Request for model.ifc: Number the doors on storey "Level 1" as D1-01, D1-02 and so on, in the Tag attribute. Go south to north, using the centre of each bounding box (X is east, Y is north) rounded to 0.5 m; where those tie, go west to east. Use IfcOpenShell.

First a look at what the model holds.

```python
import ifcopenshell
import ifcopenshell.util.element
import ifcopenshell.util.placement

model = ifcopenshell.open("model.ifc")
print(model.schema)
storey = next(s for s in model.by_type("IfcBuildingStorey") if s.Name == "Level 1")
doors = [e for e in ifcopenshell.util.element.get_decomposition(storey) if e.is_a("IfcDoor")]
for e in sorted(doors, key=lambda e: e.id()):
    origin = ifcopenshell.util.placement.get_local_placement(e.ObjectPlacement)[:3, 3]
    print(e.id(), e.Tag, e.Name, origin.round(2) + 0.0, sep=" | ")
```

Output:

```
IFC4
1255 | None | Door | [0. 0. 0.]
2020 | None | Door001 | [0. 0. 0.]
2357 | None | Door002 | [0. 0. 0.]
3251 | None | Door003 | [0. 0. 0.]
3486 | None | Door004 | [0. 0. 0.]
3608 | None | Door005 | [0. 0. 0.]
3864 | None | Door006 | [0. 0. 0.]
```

```python
import ifcopenshell
import ifcopenshell.geom
import ifcopenshell.util.element
import ifcopenshell.util.shape

model = ifcopenshell.open("model.ifc")
settings = ifcopenshell.geom.settings()
settings.set("use-world-coords", True)


def centre(element):
    shape = ifcopenshell.geom.create_shape(settings, element)
    return ifcopenshell.util.shape.get_bbox_centroid(shape.geometry)


storey = next(s for s in model.by_type("IfcBuildingStorey") if s.Name == "Level 1")
doors = [e for e in ifcopenshell.util.element.get_decomposition(storey) if e.is_a("IfcDoor")]

# Insertion points can sit at a corner or the storey origin, so sort by the geometry (in metres).
centres = {e: centre(e) for e in doors}
doors.sort(key=lambda e: (round(centres[e][1] / 0.5), centres[e][0]))

for i, e in enumerate(doors, start=1):
    number = f"D1-{i:02d}"
    e.Tag = number
    print(e.id(), number)

model.write("model_v2.ifc")
```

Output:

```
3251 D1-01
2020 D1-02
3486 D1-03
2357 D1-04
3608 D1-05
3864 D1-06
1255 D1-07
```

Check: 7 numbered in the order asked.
